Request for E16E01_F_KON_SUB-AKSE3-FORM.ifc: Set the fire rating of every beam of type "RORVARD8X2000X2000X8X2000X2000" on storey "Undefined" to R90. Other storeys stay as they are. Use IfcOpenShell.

First a look at what the model holds.

```python
import ifcopenshell
import ifcopenshell.util.element

model = ifcopenshell.open("E16E01_F_KON_SUB-AKSE3-FORM.ifc")
print(model.schema)
storey = next(s for s in model.by_type("IfcBuildingStorey") if s.Name == "Undefined")
beams = [e for e in ifcopenshell.util.element.get_decomposition(storey) if e.is_a("IfcBeam")]
seen = {}
for e in beams:
    element_type = ifcopenshell.util.element.get_type(e)
    key = (element_type.Name if element_type != e and element_type else None, ifcopenshell.util.element.get_pset(e, "Pset_BeamCommon", "FireRating"))
    seen[key] = seen.get(key, 0) + 1
for (name, value), count in sorted(seen.items(), key=str):
    print(count, "x", name, "|", value)
```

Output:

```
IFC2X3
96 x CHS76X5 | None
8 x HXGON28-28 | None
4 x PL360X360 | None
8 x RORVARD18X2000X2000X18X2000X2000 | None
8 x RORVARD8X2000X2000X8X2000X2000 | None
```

```python
import ifcopenshell
import ifcopenshell.api.pset
import ifcopenshell.util.element

model = ifcopenshell.open("E16E01_F_KON_SUB-AKSE3-FORM.ifc")

storey = next(s for s in model.by_type("IfcBuildingStorey") if s.Name == "Undefined")
beams = [e for e in ifcopenshell.util.element.get_decomposition(storey) if e.is_a("IfcBeam")]

count = 0
for e in beams:
    element_type = ifcopenshell.util.element.get_type(e)
    if element_type in (None, e) or element_type.Name != "RORVARD8X2000X2000X8X2000X2000":
        continue
    found = ifcopenshell.util.element.get_pset(e, "Pset_BeamCommon", should_inherit=False)
    if found:
        pset = model.by_id(found["id"])
        if len(ifcopenshell.util.element.get_elements_by_pset(pset)) > 1:
            pset = ifcopenshell.api.pset.unshare_pset(model, products=[e], pset=pset)[0]
    else:
        pset = ifcopenshell.api.pset.add_pset(model, product=e, name="Pset_BeamCommon")
    ifcopenshell.api.pset.edit_pset(model, pset=pset, properties={"FireRating": "R90"})
    count += 1

print(count, "beams updated")

model.write("E16E01_F_KON_SUB-AKSE3-FORM_v2.ifc")
```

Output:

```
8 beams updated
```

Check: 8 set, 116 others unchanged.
